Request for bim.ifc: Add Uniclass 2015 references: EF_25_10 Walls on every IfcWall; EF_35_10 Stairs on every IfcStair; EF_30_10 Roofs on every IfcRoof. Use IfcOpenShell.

First a look at what the model holds.

```python
import ifcopenshell

model = ifcopenshell.open("bim.ifc")
print(model.schema)
print("classifications:", [c.Name for c in model.by_type("IfcClassification")])
for ifc_class in ("IfcDoor", "IfcRoof", "IfcStair", "IfcWall", "IfcWindow"):
    print(ifc_class, len(model.by_type(ifc_class)))
```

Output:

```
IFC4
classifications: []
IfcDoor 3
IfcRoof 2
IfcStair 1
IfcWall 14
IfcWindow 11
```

```python
import ifcopenshell
import ifcopenshell.api.classification

model = ifcopenshell.open("bim.ifc")

system = ifcopenshell.api.classification.add_classification(model, classification="Uniclass 2015")

codes = {
    "IfcWall": ("EF_25_10", "Walls"),
    "IfcStair": ("EF_35_10", "Stairs"),
    "IfcRoof": ("EF_30_10", "Roofs"),
}
for ifc_class, (code, name) in codes.items():
    products = model.by_type(ifc_class)
    ifcopenshell.api.classification.add_reference(
        model, products=products, classification=system, identification=code, name=name
    )
    print(code, len(products))

model.write("bim_v2.ifc")
```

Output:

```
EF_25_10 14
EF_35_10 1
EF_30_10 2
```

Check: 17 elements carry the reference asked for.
